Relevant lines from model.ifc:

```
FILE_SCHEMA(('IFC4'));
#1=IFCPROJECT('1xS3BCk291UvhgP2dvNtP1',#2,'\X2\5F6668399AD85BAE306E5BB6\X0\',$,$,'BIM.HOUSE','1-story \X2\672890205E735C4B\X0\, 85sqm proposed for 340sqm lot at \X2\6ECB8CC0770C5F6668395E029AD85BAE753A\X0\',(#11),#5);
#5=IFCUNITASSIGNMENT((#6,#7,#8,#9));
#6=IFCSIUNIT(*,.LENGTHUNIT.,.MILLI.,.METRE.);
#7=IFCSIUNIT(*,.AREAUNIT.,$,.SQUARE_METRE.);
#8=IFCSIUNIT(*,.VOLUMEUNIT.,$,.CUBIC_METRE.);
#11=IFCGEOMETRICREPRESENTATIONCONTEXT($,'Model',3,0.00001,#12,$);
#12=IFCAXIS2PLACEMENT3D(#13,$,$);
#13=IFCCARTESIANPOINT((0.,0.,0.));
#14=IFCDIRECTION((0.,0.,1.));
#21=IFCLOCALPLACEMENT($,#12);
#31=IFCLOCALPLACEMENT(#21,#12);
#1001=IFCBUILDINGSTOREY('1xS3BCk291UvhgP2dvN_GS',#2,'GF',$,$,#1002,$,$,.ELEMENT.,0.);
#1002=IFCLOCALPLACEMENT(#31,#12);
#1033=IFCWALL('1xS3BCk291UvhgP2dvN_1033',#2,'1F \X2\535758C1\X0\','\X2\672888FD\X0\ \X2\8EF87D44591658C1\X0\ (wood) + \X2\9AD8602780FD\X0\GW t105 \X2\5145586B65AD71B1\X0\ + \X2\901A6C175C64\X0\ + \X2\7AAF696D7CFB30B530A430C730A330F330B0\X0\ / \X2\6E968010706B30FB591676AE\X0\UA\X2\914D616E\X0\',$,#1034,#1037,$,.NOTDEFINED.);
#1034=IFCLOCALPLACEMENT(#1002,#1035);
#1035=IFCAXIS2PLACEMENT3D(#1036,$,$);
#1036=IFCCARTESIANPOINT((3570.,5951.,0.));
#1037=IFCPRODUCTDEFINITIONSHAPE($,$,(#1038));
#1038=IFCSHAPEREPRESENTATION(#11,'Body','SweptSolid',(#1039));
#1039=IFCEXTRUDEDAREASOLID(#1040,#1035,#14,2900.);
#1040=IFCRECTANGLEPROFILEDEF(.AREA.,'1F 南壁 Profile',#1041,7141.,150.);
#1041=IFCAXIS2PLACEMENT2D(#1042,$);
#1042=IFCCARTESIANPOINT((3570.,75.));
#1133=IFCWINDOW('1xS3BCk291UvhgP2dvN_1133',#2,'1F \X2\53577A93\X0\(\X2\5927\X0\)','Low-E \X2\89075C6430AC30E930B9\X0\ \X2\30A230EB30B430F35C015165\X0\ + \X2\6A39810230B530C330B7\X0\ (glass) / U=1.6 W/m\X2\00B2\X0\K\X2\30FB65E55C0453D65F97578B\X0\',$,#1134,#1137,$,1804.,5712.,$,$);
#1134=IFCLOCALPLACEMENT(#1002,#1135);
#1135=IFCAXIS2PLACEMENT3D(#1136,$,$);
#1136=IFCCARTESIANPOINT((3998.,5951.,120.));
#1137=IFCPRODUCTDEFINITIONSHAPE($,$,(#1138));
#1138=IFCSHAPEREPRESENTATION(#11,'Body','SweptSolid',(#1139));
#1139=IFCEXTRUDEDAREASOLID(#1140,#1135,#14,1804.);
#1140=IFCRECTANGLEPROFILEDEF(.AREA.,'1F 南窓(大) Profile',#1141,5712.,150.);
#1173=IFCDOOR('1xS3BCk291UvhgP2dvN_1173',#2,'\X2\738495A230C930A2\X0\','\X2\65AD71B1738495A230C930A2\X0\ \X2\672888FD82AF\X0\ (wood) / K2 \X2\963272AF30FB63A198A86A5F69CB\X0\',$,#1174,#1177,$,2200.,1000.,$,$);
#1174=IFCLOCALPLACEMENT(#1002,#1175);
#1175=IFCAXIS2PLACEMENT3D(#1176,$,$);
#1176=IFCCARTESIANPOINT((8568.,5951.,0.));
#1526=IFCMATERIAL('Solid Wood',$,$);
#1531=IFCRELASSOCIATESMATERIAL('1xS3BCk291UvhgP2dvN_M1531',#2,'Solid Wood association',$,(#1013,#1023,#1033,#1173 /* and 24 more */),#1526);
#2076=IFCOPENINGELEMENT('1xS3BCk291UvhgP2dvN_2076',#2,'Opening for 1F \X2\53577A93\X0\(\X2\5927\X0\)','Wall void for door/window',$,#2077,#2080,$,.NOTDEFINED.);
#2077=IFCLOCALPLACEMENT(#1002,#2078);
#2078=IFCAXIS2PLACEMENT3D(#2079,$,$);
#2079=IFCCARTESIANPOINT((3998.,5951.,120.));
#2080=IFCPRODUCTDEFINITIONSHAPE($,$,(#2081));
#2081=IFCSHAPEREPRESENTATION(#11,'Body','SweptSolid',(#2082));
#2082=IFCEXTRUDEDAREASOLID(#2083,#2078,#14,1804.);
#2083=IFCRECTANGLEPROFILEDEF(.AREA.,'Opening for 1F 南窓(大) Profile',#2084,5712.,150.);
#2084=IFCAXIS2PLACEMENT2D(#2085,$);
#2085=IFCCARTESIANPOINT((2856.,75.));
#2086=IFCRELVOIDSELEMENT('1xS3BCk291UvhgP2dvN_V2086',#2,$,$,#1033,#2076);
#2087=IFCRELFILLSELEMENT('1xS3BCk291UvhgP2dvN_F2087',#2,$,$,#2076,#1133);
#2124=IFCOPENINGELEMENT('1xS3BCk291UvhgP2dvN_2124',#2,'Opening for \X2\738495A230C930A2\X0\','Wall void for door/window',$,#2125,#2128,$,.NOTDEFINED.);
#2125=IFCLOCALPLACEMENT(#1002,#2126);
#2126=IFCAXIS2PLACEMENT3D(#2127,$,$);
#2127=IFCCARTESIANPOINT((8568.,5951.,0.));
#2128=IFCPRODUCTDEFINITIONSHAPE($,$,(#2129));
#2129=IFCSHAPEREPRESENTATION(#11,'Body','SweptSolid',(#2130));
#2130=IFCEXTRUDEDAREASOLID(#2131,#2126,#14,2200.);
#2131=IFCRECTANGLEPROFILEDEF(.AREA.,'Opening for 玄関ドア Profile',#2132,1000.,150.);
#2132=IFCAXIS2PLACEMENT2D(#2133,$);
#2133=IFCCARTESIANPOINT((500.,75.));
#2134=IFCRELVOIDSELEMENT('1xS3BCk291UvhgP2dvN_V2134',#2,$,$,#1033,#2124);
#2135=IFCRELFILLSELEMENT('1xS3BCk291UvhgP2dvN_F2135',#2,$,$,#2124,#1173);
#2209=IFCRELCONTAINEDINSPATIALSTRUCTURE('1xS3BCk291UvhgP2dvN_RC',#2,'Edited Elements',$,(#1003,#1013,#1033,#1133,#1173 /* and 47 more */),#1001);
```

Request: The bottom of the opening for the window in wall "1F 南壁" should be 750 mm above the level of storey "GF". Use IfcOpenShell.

```python
import numpy as np
import ifcopenshell
import ifcopenshell.api.geometry
import ifcopenshell.geom
import ifcopenshell.util.element
import ifcopenshell.util.placement
import ifcopenshell.util.shape
import ifcopenshell.util.unit

model = ifcopenshell.open("model.ifc")
unit_scale = ifcopenshell.util.unit.calculate_unit_scale(model)

window = model.by_guid("1xS3BCk291UvhgP2dvN_1133")
opening = window.FillsVoids[0].RelatingOpeningElement
storey = ifcopenshell.util.element.get_container(window, ifc_class="IfcBuildingStorey")
level = ifcopenshell.util.placement.get_local_placement(storey.ObjectPlacement)[2, 3]

# The opening's origin need not be at the sill, so measure its lowest point.
shape = ifcopenshell.geom.create_shape(ifcopenshell.geom.settings(), opening)
bottom = ifcopenshell.util.shape.get_shape_bottom_elevation(shape, shape.geometry) / unit_scale
dz = level + 0.75 / unit_scale - bottom

shift = np.array([0.0, 0.0, dz])
# The window is not placed relative to its opening, so move both.
for product in (opening, window):
    matrix = ifcopenshell.util.placement.get_local_placement(product.ObjectPlacement)
    matrix[:3, 3] += shift
    ifcopenshell.api.geometry.edit_object_placement(model, product=product, matrix=matrix, is_si=False)

print(f"moved by {dz * unit_scale:+.3f} m")

model.write("model_edited.ifc")
```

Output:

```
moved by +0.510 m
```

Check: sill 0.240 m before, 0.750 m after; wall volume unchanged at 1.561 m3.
